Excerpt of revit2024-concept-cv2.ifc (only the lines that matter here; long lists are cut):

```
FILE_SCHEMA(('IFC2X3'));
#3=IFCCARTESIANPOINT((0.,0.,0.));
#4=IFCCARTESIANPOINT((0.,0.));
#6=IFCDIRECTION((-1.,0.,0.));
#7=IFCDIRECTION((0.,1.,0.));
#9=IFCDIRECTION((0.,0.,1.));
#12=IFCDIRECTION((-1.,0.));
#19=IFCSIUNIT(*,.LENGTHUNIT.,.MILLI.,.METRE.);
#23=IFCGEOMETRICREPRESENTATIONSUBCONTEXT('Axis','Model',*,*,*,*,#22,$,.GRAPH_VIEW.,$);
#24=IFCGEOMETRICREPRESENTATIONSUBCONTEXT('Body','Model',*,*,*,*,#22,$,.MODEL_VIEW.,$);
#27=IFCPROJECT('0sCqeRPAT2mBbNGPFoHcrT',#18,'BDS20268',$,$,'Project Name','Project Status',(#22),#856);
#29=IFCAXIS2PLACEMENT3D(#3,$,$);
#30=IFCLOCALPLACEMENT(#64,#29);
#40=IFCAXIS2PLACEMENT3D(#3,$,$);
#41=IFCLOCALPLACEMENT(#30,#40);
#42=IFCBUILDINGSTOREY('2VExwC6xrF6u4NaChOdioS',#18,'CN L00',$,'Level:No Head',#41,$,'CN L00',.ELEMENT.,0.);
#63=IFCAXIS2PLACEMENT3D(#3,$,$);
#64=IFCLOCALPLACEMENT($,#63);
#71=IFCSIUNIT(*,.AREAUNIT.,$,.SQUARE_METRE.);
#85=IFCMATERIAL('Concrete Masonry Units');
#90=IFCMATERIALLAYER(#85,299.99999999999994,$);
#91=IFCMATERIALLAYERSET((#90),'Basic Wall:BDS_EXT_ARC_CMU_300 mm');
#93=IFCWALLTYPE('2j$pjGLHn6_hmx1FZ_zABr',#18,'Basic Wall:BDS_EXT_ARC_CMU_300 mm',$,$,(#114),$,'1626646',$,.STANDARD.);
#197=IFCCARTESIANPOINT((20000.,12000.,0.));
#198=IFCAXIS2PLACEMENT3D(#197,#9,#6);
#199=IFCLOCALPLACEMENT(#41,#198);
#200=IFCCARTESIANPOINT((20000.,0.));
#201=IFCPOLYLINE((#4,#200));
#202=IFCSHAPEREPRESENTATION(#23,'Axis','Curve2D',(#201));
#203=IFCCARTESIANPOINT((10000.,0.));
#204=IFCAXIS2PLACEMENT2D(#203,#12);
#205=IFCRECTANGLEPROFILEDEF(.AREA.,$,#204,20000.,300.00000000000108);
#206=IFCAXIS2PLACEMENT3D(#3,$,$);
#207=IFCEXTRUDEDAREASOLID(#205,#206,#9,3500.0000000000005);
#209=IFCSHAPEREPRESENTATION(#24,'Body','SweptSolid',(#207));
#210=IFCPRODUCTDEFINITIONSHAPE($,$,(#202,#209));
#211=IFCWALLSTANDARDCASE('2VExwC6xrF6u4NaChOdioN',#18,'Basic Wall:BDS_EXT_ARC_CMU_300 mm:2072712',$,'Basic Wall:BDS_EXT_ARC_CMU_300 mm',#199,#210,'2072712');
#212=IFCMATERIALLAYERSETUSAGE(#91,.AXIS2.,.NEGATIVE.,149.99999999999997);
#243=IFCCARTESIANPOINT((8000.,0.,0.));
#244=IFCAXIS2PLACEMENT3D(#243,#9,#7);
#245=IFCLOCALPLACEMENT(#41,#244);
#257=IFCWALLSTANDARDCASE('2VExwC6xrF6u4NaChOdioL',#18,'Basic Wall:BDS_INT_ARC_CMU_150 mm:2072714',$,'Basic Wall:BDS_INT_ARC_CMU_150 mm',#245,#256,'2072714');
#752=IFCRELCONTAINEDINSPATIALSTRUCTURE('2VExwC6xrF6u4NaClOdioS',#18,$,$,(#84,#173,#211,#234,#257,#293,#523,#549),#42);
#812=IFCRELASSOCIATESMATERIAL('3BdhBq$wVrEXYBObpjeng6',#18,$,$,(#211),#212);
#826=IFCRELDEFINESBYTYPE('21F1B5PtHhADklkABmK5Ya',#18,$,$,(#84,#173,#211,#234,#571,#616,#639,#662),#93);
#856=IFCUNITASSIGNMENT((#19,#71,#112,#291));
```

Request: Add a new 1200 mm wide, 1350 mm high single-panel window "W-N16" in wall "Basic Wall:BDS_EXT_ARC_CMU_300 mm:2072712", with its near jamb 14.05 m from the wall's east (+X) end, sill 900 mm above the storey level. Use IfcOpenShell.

```python
import numpy as np
import ifcopenshell
import ifcopenshell.api.feature
import ifcopenshell.api.geometry
import ifcopenshell.api.root
import ifcopenshell.api.spatial
import ifcopenshell.api.type
import ifcopenshell.geom
import ifcopenshell.util.element
import ifcopenshell.util.placement
import ifcopenshell.util.representation
import ifcopenshell.util.shape
import ifcopenshell.util.unit

model = ifcopenshell.open("revit2024-concept-cv2.ifc")
unit_scale = ifcopenshell.util.unit.calculate_unit_scale(model)
settings = ifcopenshell.geom.settings()


def volume(element):
    """Net volume in cubic metres, openings subtracted."""
    shape = ifcopenshell.geom.create_shape(settings, element)
    return ifcopenshell.util.shape.get_volume(shape.geometry)


wall = model.by_guid("2VExwC6xrF6u4NaChOdioN")
storey = ifcopenshell.util.element.get_container(wall, ifc_class="IfcBuildingStorey")
context = ifcopenshell.util.representation.get_context(model, "Model", "Body", "MODEL_VIEW")
before = volume(wall)

width, height, from_end, sill = 1.2, 1.35, 14.05, 0.9  # metres

# The wall runs along its own X axis, and the end named is its -X end.
wall_shape = ifcopenshell.geom.create_shape(settings, wall)
x, y, z = ifcopenshell.util.shape.get_vertices(wall_shape.geometry).T
start = x.min() + from_end
face, thickness = float(y.min()), float(y.max() - y.min())
wall_matrix = ifcopenshell.util.placement.get_local_placement(wall.ObjectPlacement)
level = ifcopenshell.util.placement.get_local_placement(storey.ObjectPlacement)[2, 3]


def in_wall(x, y):
    """Placement at x, y metres in the wall's axes, at sill height."""
    matrix = wall_matrix.copy()
    matrix[:, 3] = wall_matrix @ np.array([x / unit_scale, y / unit_scale, 0.0, 1.0])
    matrix[2, 3] = level + sill / unit_scale
    return matrix


# Opening: a box that overshoots both wall faces by 50 mm.
opening = ifcopenshell.api.root.create_entity(model, ifc_class="IfcOpeningElement")
box = ifcopenshell.api.geometry.add_wall_representation(
    model, context=context, length=width, height=height, thickness=thickness + 0.1
)
ifcopenshell.api.geometry.assign_representation(model, product=opening, representation=box)
ifcopenshell.api.geometry.edit_object_placement(model, product=opening, matrix=in_wall(start, face - 0.05), is_si=False)
ifcopenshell.api.feature.add_feature(model, feature=opening, element=wall)

window = ifcopenshell.api.root.create_entity(model, ifc_class="IfcWindow", name="W-N16")
window.OverallWidth, window.OverallHeight = width / unit_scale, height / unit_scale
body = ifcopenshell.api.geometry.add_window_representation(
    model,
    context=context,
    overall_width=window.OverallWidth,
    overall_height=window.OverallHeight,
    partition_type="SINGLE_PANEL",
)
ifcopenshell.api.geometry.assign_representation(model, product=window, representation=body)
ifcopenshell.api.spatial.assign_container(model, products=[window], relating_structure=storey)
fills = ifcopenshell.api.feature.add_filling(model, opening=opening, element=window)
fills.OwnerHistory = window.OwnerHistory  # required in IFC2X3

# IFC2X3 keeps the operation on the window style.
style = ifcopenshell.api.root.create_entity(model, ifc_class="IfcWindowStyle", name="W-N16")
style.OperationType, style.ConstructionType = "SINGLE_PANEL", "NOTDEFINED"
style.ParameterTakesPrecedence = style.Sizeable = False
ifcopenshell.api.type.assign_type(model, related_objects=[window], relating_type=style)

# Centre the window in the wall's thickness.
ifcopenshell.api.geometry.edit_object_placement(model, product=window, matrix=in_wall(start, face), is_si=False)
window_shape = ifcopenshell.geom.create_shape(settings, window)
depth = ifcopenshell.util.shape.get_vertices(window_shape.geometry)[:, 1]
offset = face + thickness / 2 - (depth.min() + depth.max()) / 2
ifcopenshell.api.geometry.edit_object_placement(model, product=window, matrix=in_wall(start, offset), is_si=False)

after = volume(wall)

print(f"wall volume {before:.3f} -> {after:.3f} m3")

model.write("revit2024-concept-cv2_updated.ifc")
```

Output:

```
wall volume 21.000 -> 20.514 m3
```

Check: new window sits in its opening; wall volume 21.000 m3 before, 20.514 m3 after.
